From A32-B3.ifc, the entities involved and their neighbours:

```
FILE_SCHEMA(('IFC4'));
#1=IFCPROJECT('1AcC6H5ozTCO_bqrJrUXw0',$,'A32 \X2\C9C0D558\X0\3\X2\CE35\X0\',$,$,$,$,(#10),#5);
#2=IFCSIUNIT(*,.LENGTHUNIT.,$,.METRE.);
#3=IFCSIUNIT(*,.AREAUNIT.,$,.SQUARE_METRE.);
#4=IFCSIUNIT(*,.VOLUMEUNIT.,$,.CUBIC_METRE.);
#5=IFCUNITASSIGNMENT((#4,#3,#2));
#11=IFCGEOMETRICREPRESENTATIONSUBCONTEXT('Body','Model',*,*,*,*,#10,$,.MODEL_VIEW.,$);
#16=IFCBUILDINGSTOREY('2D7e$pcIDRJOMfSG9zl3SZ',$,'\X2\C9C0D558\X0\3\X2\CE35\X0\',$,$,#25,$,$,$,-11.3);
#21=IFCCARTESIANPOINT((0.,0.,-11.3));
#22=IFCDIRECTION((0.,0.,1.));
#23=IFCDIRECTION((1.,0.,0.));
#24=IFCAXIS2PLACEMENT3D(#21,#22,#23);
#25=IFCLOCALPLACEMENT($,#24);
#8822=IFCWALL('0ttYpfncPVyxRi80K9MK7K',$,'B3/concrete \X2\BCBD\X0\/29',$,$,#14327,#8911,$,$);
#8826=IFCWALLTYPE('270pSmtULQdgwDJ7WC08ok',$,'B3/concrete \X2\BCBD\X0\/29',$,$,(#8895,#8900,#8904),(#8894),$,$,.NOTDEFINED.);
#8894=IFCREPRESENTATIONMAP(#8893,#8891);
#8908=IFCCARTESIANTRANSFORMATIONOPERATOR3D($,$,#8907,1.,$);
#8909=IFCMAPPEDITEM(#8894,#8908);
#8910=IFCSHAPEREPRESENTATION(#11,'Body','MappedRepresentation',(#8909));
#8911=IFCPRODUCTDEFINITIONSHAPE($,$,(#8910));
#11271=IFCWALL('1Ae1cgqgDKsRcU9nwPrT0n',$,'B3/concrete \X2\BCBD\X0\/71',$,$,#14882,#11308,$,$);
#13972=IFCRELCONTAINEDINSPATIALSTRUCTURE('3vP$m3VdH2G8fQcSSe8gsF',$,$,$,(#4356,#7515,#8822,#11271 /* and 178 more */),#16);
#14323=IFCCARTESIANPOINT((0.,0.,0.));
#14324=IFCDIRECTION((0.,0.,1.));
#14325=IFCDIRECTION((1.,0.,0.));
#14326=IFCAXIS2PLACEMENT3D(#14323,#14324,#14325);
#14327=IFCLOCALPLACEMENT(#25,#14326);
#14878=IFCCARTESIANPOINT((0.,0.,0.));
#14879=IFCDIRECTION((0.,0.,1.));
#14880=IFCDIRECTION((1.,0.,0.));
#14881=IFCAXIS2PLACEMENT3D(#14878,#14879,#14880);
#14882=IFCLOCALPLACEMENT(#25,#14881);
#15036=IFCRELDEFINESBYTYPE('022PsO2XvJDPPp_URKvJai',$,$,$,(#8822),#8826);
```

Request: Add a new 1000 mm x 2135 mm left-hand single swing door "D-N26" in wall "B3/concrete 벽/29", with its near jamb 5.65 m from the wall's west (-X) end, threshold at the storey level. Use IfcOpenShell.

```python
import numpy as np
import ifcopenshell
import ifcopenshell.api.feature
import ifcopenshell.api.geometry
import ifcopenshell.api.root
import ifcopenshell.api.spatial
import ifcopenshell.geom
import ifcopenshell.util.element
import ifcopenshell.util.placement
import ifcopenshell.util.representation
import ifcopenshell.util.shape
import ifcopenshell.util.unit

model = ifcopenshell.open("A32-B3.ifc")
unit_scale = ifcopenshell.util.unit.calculate_unit_scale(model)
settings = ifcopenshell.geom.settings()


def volume(element):
    """Net volume in cubic metres, openings subtracted."""
    shape = ifcopenshell.geom.create_shape(settings, element)
    return ifcopenshell.util.shape.get_volume(shape.geometry)


wall = model.by_guid("0ttYpfncPVyxRi80K9MK7K")
storey = ifcopenshell.util.element.get_container(wall, ifc_class="IfcBuildingStorey")
context = ifcopenshell.util.representation.get_context(model, "Model", "Body", "MODEL_VIEW")
before = volume(wall)

width, height, from_end, sill = 1, 2.135, 5.65, 0.0  # metres

# The wall runs along its own X axis, and the end named is its -X end.
wall_shape = ifcopenshell.geom.create_shape(settings, wall)
x, y, z = ifcopenshell.util.shape.get_vertices(wall_shape.geometry).T
start = x.min() + from_end
face, thickness = float(y.min()), float(y.max() - y.min())
wall_matrix = ifcopenshell.util.placement.get_local_placement(wall.ObjectPlacement)
level = ifcopenshell.util.placement.get_local_placement(storey.ObjectPlacement)[2, 3]


def in_wall(x, y):
    """Placement at x, y metres in the wall's axes, at sill height."""
    matrix = wall_matrix.copy()
    matrix[:, 3] = wall_matrix @ np.array([x / unit_scale, y / unit_scale, 0.0, 1.0])
    matrix[2, 3] = level + sill / unit_scale
    return matrix


# Opening: a box that overshoots both wall faces by 50 mm.
opening = ifcopenshell.api.root.create_entity(model, ifc_class="IfcOpeningElement", predefined_type="OPENING")
box = ifcopenshell.api.geometry.add_wall_representation(
    model, context=context, length=width, height=height, thickness=thickness + 0.1
)
ifcopenshell.api.geometry.assign_representation(model, product=opening, representation=box)
ifcopenshell.api.geometry.edit_object_placement(model, product=opening, matrix=in_wall(start, face - 0.05), is_si=False)
ifcopenshell.api.feature.add_feature(model, feature=opening, element=wall)

door = ifcopenshell.api.root.create_entity(model, ifc_class="IfcDoor", name="D-N26", predefined_type="DOOR")
door.OverallWidth, door.OverallHeight = width / unit_scale, height / unit_scale
door.OperationType = "SINGLE_SWING_LEFT"
body = ifcopenshell.api.geometry.add_door_representation(
    model,
    context=context,
    overall_width=door.OverallWidth,
    overall_height=door.OverallHeight,
    operation_type="SINGLE_SWING_LEFT",
    lining_properties={"LiningDepth": thickness / unit_scale, "ThresholdDepth": thickness / unit_scale},
)
ifcopenshell.api.geometry.assign_representation(model, product=door, representation=body)
ifcopenshell.api.spatial.assign_container(model, products=[door], relating_structure=storey)
ifcopenshell.api.feature.add_filling(model, opening=opening, element=door)

# The lining spans the wall, so the door starts at the wall face.
ifcopenshell.api.geometry.edit_object_placement(model, product=door, matrix=in_wall(start, face), is_si=False)

after = volume(wall)

print(f"wall volume {before:.3f} -> {after:.3f} m3")

model.write("A32-B3_updated.ifc")
```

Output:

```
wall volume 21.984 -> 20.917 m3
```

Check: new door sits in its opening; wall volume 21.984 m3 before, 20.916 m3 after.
